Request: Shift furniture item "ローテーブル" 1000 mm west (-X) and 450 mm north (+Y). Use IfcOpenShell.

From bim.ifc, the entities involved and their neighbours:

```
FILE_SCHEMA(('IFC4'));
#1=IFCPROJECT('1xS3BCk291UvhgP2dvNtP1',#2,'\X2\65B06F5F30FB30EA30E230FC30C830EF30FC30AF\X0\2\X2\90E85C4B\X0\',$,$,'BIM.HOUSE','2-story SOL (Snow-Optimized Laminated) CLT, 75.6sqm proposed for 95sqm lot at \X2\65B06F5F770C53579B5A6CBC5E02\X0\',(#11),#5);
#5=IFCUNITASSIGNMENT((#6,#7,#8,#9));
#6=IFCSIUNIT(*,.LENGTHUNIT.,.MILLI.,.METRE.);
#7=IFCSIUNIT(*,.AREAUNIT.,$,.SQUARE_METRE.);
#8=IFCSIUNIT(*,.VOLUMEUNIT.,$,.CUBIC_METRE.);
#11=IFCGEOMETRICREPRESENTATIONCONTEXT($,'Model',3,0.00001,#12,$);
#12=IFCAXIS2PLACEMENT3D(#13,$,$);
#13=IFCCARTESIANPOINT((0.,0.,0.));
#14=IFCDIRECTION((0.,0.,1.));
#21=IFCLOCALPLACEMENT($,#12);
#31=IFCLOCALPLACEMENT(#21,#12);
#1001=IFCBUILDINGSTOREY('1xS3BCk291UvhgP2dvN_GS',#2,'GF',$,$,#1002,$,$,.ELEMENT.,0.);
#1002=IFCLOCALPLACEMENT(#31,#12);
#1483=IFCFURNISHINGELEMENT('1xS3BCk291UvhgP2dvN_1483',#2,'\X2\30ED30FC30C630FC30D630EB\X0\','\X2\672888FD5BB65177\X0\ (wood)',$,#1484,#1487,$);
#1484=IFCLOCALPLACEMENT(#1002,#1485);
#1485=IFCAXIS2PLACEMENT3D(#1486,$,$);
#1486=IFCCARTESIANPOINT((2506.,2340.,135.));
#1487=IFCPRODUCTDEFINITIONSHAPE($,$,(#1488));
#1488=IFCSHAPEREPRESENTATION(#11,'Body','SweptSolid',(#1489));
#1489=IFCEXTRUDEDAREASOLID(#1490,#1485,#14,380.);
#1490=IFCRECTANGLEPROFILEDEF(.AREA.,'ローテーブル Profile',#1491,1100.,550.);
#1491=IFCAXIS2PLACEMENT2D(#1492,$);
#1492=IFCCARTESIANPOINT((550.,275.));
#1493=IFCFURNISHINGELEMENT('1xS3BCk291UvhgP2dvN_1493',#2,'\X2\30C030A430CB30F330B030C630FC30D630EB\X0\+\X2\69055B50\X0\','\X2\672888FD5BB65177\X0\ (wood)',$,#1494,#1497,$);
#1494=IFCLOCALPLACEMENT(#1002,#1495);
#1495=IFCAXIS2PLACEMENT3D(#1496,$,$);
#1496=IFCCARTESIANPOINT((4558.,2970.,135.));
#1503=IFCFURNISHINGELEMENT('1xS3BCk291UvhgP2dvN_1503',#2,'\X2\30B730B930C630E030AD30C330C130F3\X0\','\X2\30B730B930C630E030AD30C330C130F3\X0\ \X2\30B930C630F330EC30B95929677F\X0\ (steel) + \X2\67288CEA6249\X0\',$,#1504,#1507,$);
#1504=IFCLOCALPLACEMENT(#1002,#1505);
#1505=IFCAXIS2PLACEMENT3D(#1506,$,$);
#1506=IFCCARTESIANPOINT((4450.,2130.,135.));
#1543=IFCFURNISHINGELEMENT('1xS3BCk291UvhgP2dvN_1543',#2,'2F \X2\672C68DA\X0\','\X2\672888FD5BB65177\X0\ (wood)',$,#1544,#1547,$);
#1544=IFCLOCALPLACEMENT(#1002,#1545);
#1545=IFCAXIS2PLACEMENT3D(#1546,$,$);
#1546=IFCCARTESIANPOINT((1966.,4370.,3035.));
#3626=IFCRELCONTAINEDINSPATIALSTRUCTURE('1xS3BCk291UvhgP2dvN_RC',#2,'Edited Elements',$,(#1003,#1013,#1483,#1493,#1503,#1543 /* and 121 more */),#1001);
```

```python
import ifcopenshell
import ifcopenshell.api.geometry
import ifcopenshell.util.placement
import ifcopenshell.util.unit

model = ifcopenshell.open("bim.ifc")
unit_scale = ifcopenshell.util.unit.calculate_unit_scale(model)

item = model.by_id(1483)
matrix = ifcopenshell.util.placement.get_local_placement(item.ObjectPlacement)
matrix[0, 3] -= 1 / unit_scale
matrix[1, 3] += 0.45 / unit_scale
ifcopenshell.api.geometry.edit_object_placement(model, product=item, matrix=matrix, is_si=False)

print(ifcopenshell.util.placement.get_local_placement(item.ObjectPlacement).round(3) + 0.0)

model.write("bim_updated.ifc")
```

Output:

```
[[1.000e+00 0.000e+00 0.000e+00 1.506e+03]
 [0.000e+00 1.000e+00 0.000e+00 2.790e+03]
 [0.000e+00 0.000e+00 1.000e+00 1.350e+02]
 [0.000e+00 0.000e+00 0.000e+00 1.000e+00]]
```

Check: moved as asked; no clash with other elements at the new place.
